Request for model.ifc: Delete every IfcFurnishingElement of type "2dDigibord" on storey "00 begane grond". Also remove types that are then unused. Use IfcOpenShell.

First a look at what the model holds.

```python
import ifcopenshell
import ifcopenshell.util.element

model = ifcopenshell.open("model.ifc")
print(model.schema)
storey = next(s for s in model.by_type("IfcBuildingStorey") if s.Name == "00 begane grond")
furniture = [e for e in ifcopenshell.util.element.get_decomposition(storey) if e.is_a("IfcFurnishingElement")]
seen = {}
for e in furniture:
    element_type = ifcopenshell.util.element.get_type(e)
    name = element_type.Name if element_type not in (None, e) else None
    seen[name] = seen.get(name, 0) + 1
for name, count in sorted(seen.items(), key=str):
    print(count, "x", name)
```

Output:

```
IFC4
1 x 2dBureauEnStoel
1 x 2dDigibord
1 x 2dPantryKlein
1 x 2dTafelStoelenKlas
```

```python
import ifcopenshell
import ifcopenshell.api.root
import ifcopenshell.util.element

model = ifcopenshell.open("model.ifc")

storey = next(s for s in model.by_type("IfcBuildingStorey") if s.Name == "00 begane grond")
furniture = [e for e in ifcopenshell.util.element.get_decomposition(storey) if e.is_a("IfcFurnishingElement")]
targets = [e for e in furniture if (t := ifcopenshell.util.element.get_type(e)) not in (None, e) and t.Name == "2dDigibord"]
types = {ifcopenshell.util.element.get_type(e) for e in targets} - {None, *targets}

for e in targets:
    ifcopenshell.api.root.remove_product(model, product=e)
print(len(targets), "removed")

unused = [t for t in types if not ifcopenshell.util.element.get_types(t)]
for t in unused:
    ifcopenshell.api.root.remove_product(model, product=t)
print(len(unused), "unused types removed")

model.write("model_rev.ifc")
```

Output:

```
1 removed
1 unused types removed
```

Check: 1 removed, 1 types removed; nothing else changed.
